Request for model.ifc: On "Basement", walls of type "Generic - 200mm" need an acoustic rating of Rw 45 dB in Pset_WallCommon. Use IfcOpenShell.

First a look at what the model holds.

```python
import ifcopenshell
import ifcopenshell.util.element

model = ifcopenshell.open("model.ifc")
print(model.schema)
storey = next(s for s in model.by_type("IfcBuildingStorey") if s.Name == "Basement")
walls = [e for e in ifcopenshell.util.element.get_decomposition(storey) if e.is_a("IfcWall")]
seen = {}
for e in walls:
    element_type = ifcopenshell.util.element.get_type(e)
    key = (element_type.Name if element_type != e and element_type else None, ifcopenshell.util.element.get_pset(e, "Pset_WallCommon", "AcousticRating"))
    seen[key] = seen.get(key, 0) + 1
for (name, value), count in sorted(seen.items(), key=str):
    print(count, "x", name, "|", value)
```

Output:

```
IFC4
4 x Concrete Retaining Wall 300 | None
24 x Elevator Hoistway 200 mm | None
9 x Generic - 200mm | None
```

```python
import ifcopenshell
import ifcopenshell.api.pset
import ifcopenshell.util.element

model = ifcopenshell.open("model.ifc")

storey = next(s for s in model.by_type("IfcBuildingStorey") if s.Name == "Basement")
walls = [e for e in ifcopenshell.util.element.get_decomposition(storey) if e.is_a("IfcWall")]

count = 0
for e in walls:
    element_type = ifcopenshell.util.element.get_type(e)
    if element_type in (None, e) or element_type.Name != "Generic - 200mm":
        continue
    # add_pset returns the element's existing set when there is one.
    pset = ifcopenshell.api.pset.add_pset(model, product=e, name="Pset_WallCommon")
    ifcopenshell.api.pset.edit_pset(model, pset=pset, properties={"AcousticRating": "Rw 45 dB"})
    count += 1

print(count, "walls updated")

model.write("model_v2.ifc")
```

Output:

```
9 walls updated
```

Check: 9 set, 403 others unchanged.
